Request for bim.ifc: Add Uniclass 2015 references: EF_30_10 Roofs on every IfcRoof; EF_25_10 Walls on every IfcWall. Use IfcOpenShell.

First a look at what the model holds.

```python
import ifcopenshell

model = ifcopenshell.open("bim.ifc")
print(model.schema)
print("classifications:", [c.Name for c in model.by_type("IfcClassification")])
for ifc_class in ("IfcDoor", "IfcRoof", "IfcStair", "IfcWall", "IfcWindow"):
    print(ifc_class, len(model.by_type(ifc_class)))
```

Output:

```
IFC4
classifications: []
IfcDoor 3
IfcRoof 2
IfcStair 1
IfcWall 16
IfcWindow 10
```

```python
import ifcopenshell
import ifcopenshell.api.classification

model = ifcopenshell.open("bim.ifc")

system = ifcopenshell.api.classification.add_classification(model, classification="Uniclass 2015")

codes = {
    "IfcRoof": ("EF_30_10", "Roofs"),
    "IfcWall": ("EF_25_10", "Walls"),
}
for ifc_class, (code, name) in codes.items():
    products = model.by_type(ifc_class)
    ifcopenshell.api.classification.add_reference(
        model, products=products, classification=system, identification=code, name=name
    )
    print(code, len(products))

model.write("bim-out.ifc")
```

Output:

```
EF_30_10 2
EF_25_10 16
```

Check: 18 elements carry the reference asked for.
